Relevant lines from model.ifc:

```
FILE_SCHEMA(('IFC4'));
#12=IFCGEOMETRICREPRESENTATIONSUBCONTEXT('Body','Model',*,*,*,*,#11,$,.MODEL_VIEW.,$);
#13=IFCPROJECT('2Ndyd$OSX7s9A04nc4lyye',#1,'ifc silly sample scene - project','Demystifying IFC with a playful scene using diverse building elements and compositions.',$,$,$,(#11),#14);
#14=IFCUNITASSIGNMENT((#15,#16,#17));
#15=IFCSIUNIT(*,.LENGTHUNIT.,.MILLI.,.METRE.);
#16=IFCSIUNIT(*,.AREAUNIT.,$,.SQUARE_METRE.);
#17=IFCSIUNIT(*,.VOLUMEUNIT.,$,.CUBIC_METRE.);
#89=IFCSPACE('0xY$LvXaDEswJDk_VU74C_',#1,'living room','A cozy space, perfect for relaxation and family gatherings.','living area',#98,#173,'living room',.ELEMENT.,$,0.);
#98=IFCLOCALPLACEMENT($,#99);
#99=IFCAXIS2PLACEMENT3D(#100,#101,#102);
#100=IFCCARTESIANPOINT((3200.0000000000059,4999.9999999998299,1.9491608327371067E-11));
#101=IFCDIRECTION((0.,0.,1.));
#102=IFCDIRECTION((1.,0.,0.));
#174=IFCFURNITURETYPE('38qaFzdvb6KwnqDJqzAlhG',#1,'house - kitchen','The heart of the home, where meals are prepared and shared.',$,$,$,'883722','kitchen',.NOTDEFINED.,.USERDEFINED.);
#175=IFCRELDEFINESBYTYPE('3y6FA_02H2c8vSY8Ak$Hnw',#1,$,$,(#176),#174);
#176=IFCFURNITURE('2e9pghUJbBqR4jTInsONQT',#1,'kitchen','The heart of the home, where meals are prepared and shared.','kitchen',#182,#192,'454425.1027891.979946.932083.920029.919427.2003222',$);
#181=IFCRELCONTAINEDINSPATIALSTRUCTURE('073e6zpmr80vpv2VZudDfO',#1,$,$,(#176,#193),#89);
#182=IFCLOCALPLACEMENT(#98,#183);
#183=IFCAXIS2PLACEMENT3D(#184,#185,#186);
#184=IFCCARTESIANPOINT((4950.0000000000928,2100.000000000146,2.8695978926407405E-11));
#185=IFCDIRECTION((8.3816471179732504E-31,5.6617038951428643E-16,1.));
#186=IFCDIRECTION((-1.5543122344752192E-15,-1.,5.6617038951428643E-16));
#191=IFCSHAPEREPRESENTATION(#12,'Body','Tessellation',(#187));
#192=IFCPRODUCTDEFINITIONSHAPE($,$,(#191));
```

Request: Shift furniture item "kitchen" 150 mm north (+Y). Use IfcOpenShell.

```python
import ifcopenshell
import ifcopenshell.api.geometry
import ifcopenshell.util.placement
import ifcopenshell.util.unit

model = ifcopenshell.open("model.ifc")
unit_scale = ifcopenshell.util.unit.calculate_unit_scale(model)

item = model.by_guid("2e9pghUJbBqR4jTInsONQT")
matrix = ifcopenshell.util.placement.get_local_placement(item.ObjectPlacement)
matrix[1, 3] += 0.15 / unit_scale
ifcopenshell.api.geometry.edit_object_placement(model, product=item, matrix=matrix, is_si=False)

print(ifcopenshell.util.placement.get_local_placement(item.ObjectPlacement).round(3) + 0.0)

model.write("model_updated.ifc")
```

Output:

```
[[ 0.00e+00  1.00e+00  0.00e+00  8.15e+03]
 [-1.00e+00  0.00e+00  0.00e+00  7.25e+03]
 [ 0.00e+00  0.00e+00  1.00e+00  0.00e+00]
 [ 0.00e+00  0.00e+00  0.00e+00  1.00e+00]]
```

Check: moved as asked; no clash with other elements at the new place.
